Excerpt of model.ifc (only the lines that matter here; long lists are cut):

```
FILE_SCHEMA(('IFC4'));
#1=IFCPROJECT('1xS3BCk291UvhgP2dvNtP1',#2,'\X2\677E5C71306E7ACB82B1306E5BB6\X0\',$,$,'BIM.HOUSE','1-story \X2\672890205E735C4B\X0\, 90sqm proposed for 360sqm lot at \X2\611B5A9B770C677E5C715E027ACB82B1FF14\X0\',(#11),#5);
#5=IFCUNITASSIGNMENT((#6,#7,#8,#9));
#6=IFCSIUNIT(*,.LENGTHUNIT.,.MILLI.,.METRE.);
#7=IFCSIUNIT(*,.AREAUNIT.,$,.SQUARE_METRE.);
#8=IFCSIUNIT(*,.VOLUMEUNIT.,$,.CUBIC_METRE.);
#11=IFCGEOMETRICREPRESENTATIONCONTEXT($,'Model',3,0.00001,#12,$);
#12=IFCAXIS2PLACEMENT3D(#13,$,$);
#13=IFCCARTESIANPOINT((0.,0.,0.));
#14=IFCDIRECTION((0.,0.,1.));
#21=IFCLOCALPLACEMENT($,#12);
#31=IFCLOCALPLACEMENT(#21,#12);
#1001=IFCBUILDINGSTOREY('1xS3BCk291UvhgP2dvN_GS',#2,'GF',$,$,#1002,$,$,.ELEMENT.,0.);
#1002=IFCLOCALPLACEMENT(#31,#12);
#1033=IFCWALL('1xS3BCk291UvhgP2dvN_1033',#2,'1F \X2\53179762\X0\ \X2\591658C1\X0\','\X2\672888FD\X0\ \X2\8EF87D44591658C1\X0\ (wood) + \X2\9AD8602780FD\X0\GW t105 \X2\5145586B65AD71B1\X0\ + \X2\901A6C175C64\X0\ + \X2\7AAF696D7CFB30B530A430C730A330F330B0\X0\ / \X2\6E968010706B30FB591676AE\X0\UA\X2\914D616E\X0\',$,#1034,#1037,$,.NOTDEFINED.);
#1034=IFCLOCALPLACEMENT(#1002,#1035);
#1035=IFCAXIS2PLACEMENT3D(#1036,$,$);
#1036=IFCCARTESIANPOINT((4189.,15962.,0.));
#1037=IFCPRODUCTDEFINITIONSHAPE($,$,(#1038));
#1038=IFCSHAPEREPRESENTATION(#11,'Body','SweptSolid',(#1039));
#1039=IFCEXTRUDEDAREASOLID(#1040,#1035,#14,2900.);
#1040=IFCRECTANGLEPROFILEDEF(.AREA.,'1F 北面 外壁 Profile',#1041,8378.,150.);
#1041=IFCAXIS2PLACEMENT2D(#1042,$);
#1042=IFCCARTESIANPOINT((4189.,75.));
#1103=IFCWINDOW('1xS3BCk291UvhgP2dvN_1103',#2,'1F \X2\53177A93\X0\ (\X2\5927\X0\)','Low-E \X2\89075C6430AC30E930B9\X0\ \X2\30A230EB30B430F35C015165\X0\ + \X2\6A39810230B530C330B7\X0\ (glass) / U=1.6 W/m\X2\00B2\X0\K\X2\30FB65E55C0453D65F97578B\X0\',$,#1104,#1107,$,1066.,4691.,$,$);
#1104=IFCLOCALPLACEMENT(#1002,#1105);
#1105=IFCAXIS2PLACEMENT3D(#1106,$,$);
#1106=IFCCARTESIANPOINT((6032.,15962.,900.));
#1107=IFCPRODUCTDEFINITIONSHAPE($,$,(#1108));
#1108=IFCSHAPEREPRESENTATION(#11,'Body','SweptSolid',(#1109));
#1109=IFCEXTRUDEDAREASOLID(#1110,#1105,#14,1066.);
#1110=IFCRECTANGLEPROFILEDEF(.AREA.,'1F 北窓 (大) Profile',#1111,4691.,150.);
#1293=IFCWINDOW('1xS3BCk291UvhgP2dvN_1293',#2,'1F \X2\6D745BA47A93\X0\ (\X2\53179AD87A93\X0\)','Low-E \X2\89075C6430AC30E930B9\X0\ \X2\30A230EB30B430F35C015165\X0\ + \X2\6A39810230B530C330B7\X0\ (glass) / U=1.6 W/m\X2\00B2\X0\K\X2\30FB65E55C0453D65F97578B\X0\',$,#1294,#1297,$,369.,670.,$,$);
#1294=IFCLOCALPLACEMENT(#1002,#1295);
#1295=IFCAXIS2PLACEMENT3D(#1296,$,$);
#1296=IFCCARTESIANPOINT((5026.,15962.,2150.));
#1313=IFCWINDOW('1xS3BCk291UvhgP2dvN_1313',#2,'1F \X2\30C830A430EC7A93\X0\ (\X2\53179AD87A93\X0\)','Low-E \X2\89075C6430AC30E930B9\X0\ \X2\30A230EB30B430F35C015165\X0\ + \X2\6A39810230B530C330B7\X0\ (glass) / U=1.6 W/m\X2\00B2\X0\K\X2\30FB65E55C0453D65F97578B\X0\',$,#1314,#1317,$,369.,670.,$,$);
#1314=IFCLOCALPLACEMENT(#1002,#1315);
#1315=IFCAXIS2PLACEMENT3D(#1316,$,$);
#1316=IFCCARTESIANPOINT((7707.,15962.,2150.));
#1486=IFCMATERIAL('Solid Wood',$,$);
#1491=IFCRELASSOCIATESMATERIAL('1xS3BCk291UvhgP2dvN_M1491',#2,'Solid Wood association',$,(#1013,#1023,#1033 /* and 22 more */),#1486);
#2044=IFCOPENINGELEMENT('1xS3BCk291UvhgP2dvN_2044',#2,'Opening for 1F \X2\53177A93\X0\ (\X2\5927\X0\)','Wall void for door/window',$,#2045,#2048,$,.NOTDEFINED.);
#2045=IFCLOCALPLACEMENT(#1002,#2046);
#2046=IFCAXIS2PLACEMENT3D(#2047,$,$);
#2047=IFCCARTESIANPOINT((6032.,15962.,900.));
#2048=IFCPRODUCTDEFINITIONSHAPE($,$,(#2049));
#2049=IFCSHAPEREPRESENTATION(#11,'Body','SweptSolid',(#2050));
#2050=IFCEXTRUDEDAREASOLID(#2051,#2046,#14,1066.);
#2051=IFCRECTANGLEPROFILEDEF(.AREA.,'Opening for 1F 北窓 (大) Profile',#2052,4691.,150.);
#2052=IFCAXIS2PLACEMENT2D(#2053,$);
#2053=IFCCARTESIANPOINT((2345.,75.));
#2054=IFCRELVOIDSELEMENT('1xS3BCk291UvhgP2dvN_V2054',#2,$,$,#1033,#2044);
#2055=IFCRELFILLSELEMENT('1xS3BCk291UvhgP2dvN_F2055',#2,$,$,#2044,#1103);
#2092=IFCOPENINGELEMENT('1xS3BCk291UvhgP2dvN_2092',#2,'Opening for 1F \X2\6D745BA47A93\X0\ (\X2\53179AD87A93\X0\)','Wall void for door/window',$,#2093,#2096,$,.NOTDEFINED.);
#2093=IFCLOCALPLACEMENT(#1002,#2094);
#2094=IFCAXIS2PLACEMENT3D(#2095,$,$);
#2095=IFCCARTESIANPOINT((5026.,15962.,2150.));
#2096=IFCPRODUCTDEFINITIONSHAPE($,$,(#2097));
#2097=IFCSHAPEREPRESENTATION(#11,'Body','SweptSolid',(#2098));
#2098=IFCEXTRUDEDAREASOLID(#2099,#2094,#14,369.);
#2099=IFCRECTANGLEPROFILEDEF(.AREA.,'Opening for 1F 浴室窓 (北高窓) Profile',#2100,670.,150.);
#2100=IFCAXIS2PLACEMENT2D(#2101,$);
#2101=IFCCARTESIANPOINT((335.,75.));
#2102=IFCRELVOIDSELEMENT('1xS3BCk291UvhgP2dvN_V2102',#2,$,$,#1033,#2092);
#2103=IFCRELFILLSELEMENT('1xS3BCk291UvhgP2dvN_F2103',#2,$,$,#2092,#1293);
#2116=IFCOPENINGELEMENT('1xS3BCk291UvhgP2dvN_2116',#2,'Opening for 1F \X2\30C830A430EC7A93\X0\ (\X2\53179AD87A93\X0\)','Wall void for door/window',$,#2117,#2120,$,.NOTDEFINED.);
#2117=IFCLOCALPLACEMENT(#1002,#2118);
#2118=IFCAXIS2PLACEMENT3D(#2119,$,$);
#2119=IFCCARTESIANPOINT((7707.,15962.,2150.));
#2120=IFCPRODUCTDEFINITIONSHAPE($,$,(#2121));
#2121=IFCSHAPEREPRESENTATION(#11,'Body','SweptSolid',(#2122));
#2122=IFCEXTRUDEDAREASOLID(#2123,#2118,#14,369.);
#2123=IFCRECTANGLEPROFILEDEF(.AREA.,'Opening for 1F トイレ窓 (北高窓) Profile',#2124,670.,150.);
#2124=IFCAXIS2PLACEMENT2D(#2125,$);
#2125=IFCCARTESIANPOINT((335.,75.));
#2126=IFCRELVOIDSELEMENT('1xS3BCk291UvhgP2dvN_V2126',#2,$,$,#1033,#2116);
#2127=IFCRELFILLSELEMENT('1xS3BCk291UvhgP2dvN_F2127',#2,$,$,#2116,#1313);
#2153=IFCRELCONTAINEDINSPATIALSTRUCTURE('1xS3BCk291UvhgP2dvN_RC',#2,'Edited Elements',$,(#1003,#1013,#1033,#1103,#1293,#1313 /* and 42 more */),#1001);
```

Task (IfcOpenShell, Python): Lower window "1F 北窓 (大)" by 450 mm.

```python
import numpy as np
import ifcopenshell
import ifcopenshell.api.geometry
import ifcopenshell.util.placement
import ifcopenshell.util.unit

model = ifcopenshell.open("model.ifc")
unit_scale = ifcopenshell.util.unit.calculate_unit_scale(model)

window = model.by_id(1103)
opening = window.FillsVoids[0].RelatingOpeningElement
dz = -450.0

shift = np.array([0.0, 0.0, dz])
# The window is not placed relative to its opening, so move both.
for product in (opening, window):
    matrix = ifcopenshell.util.placement.get_local_placement(product.ObjectPlacement)
    matrix[:3, 3] += shift
    ifcopenshell.api.geometry.edit_object_placement(model, product=product, matrix=matrix, is_si=False)

print(f"moved by {dz * unit_scale:+.3f} m")

model.write("model_rev.ifc")
```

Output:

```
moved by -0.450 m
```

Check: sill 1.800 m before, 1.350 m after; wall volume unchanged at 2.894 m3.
